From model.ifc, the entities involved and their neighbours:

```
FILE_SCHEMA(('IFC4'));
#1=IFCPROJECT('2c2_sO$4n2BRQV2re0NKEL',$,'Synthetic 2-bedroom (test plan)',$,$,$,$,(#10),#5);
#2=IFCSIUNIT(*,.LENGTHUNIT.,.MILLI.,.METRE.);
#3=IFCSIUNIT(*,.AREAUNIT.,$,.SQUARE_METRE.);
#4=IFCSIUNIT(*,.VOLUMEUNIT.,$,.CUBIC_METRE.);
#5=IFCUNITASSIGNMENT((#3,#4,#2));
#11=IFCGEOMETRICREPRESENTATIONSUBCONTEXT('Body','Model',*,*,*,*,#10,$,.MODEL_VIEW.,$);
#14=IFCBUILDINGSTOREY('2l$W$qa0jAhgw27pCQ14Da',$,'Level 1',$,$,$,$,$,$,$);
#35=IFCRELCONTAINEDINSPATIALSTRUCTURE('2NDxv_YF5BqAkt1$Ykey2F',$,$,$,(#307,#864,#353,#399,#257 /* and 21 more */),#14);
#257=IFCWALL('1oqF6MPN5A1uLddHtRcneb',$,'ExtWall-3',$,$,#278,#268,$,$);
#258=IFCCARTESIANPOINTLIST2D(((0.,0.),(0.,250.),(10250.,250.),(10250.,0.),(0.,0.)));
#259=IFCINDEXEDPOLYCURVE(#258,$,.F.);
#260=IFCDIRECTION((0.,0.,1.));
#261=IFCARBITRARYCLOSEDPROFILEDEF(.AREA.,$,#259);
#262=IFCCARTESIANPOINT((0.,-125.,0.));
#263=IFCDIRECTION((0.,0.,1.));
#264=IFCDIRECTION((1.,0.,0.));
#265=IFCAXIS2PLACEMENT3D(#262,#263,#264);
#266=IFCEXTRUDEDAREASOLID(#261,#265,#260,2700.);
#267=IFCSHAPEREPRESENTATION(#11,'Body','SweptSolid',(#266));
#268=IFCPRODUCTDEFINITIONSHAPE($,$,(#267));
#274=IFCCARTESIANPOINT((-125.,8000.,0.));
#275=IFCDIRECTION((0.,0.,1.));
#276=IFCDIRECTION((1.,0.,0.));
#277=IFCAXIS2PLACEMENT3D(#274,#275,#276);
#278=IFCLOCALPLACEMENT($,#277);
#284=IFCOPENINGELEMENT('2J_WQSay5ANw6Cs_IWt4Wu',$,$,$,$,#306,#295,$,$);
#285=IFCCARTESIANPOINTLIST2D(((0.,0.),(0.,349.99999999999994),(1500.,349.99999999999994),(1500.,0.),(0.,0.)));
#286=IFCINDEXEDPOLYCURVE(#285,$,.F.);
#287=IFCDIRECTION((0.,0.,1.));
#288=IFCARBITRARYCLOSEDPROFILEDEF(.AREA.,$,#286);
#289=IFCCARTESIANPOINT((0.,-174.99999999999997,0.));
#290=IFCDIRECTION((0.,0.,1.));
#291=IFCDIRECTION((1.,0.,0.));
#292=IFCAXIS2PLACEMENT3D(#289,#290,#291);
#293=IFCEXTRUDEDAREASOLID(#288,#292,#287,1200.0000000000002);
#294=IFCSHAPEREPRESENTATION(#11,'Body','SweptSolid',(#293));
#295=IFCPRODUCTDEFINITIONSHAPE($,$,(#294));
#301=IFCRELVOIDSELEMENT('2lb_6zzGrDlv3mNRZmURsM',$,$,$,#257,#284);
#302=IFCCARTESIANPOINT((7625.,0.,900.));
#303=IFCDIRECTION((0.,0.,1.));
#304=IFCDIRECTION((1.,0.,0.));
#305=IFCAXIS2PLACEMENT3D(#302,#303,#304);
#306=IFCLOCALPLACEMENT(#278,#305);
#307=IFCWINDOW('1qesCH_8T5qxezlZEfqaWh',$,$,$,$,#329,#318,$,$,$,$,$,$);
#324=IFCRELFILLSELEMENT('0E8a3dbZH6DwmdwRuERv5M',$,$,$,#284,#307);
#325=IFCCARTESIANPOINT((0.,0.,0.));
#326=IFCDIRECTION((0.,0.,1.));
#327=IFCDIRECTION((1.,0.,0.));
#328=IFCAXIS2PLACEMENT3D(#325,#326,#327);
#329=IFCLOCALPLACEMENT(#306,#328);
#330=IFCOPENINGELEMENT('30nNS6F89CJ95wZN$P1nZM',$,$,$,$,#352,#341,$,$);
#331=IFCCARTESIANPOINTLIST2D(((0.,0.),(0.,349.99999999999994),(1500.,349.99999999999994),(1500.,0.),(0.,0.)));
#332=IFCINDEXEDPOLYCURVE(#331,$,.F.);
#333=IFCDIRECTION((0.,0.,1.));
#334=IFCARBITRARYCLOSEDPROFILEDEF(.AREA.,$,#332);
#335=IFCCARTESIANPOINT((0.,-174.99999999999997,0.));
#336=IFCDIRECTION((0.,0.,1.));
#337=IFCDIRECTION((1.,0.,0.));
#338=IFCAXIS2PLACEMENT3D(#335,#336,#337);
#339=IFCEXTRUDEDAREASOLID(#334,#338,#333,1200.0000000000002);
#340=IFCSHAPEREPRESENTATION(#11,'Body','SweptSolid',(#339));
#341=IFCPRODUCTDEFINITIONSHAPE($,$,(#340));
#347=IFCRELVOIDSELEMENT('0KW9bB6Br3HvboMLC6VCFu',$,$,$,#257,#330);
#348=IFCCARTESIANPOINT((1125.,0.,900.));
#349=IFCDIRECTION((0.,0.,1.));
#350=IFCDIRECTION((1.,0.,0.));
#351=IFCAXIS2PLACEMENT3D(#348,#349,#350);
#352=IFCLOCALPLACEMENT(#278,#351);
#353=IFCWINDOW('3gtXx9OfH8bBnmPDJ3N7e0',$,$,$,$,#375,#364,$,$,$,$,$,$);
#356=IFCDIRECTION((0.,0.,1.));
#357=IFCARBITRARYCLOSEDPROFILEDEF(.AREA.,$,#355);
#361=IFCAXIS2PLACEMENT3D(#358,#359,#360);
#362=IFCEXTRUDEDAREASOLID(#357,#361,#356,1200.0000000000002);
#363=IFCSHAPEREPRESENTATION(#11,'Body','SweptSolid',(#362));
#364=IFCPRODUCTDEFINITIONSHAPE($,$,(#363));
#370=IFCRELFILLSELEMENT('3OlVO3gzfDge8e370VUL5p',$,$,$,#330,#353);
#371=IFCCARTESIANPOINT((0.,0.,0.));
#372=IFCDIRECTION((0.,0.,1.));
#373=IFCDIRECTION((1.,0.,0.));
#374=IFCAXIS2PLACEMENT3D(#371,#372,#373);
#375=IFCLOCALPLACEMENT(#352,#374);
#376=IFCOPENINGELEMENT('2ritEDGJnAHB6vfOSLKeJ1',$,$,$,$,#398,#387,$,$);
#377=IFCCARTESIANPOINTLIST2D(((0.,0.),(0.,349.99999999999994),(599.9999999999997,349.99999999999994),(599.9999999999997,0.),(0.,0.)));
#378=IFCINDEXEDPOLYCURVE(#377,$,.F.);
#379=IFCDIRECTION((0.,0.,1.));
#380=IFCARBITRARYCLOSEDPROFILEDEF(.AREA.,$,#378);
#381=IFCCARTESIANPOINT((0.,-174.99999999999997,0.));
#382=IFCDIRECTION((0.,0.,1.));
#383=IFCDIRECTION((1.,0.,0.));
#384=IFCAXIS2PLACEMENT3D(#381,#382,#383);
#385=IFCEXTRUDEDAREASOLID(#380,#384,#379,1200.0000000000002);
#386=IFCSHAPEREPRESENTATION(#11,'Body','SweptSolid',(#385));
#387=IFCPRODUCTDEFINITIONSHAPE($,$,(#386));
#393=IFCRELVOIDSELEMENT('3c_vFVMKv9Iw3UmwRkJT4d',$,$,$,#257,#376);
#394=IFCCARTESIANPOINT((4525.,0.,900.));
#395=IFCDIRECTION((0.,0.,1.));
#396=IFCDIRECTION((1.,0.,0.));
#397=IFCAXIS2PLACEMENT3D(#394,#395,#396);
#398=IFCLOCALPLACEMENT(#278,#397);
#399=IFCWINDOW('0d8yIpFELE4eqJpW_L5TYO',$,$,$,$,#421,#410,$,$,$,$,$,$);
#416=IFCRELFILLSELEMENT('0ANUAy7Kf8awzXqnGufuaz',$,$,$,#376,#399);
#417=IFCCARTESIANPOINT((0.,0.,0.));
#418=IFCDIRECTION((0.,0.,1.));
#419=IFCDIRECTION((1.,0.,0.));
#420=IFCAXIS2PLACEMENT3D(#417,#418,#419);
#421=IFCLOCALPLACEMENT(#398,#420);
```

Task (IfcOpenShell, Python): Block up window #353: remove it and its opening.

```python
import ifcopenshell
import ifcopenshell.api.feature
import ifcopenshell.api.root
import ifcopenshell.geom
import ifcopenshell.util.shape

model = ifcopenshell.open("model.ifc")
settings = ifcopenshell.geom.settings()


def volume(element):
    """Net volume in cubic metres, openings subtracted."""
    shape = ifcopenshell.geom.create_shape(settings, element)
    return ifcopenshell.util.shape.get_volume(shape.geometry)


window = model.by_id(353)
opening = window.FillsVoids[0].RelatingOpeningElement
wall = opening.VoidsElements[0].RelatingBuildingElement
before = volume(wall)

ifcopenshell.api.root.remove_product(model, product=window)
ifcopenshell.api.feature.remove_feature(model, feature=opening)

after = volume(wall)

print(f"wall volume {before:.3f} -> {after:.3f} m3")

model.write("model_edited.ifc")
```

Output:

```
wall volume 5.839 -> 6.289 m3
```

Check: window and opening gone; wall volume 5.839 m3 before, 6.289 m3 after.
